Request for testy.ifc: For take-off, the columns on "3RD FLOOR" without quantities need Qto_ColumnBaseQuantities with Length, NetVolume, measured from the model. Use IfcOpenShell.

First a look at what the model holds.

```python
import ifcopenshell
import ifcopenshell.util.element
import ifcopenshell.util.unit

model = ifcopenshell.open("testy.ifc")
print(model.schema)
for unit_type in ("LENGTHUNIT", "AREAUNIT", "VOLUMEUNIT"):
    print(unit_type, ifcopenshell.util.unit.calculate_unit_scale(model, unit_type))
storey = next(s for s in model.by_type("IfcBuildingStorey") if s.Name == "3RD FLOOR")
columns = [e for e in ifcopenshell.util.element.get_decomposition(storey) if e.is_a("IfcColumn")]
for e in sorted(columns, key=lambda e: e.id()):
    print(e.id(), e.is_a(), e.Name, list(ifcopenshell.util.element.get_psets(e, qtos_only=True)), sep=" | ")
```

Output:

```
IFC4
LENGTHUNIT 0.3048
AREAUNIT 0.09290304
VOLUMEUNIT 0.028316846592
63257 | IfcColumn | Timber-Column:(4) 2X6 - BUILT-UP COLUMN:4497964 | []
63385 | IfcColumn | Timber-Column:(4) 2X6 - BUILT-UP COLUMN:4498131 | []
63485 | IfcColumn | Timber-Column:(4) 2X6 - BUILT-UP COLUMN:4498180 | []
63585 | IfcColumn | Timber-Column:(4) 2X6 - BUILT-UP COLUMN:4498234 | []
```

```python
import ifcopenshell
import ifcopenshell.api.pset
import ifcopenshell.geom
import ifcopenshell.util.element
import ifcopenshell.util.shape
import ifcopenshell.util.unit

model = ifcopenshell.open("testy.ifc")
unit_scale = ifcopenshell.util.unit.calculate_unit_scale(model)
volume_scale = ifcopenshell.util.unit.calculate_unit_scale(model, "VOLUMEUNIT")
settings = ifcopenshell.geom.settings()

storey = next(s for s in model.by_type("IfcBuildingStorey") if s.Name == "3RD FLOOR")
columns = [e for e in ifcopenshell.util.element.get_decomposition(storey) if e.is_a("IfcColumn")]

for e in sorted(columns, key=lambda e: e.id()):
    if ifcopenshell.util.element.get_psets(e, qtos_only=True, should_inherit=False):
        continue
    # Geometry comes back in metres, in the element's own axes.
    shape = ifcopenshell.geom.create_shape(settings, e)
    values = {
        "Length": ifcopenshell.util.shape.get_z(shape.geometry) / unit_scale,
        "NetVolume": ifcopenshell.util.shape.get_volume(shape.geometry) / volume_scale,
    }
    qto = ifcopenshell.api.pset.add_qto(model, product=e, name="Qto_ColumnBaseQuantities")
    ifcopenshell.api.pset.edit_qto(model, qto=qto, properties=values)
    print(e.id(), {k: round(v, 3) for k, v in values.items()})

model.write("testy_edited.ifc")
```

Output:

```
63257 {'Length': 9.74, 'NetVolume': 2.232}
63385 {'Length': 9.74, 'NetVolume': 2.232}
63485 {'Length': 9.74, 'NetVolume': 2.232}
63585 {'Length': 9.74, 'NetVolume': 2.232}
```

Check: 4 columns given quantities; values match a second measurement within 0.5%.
